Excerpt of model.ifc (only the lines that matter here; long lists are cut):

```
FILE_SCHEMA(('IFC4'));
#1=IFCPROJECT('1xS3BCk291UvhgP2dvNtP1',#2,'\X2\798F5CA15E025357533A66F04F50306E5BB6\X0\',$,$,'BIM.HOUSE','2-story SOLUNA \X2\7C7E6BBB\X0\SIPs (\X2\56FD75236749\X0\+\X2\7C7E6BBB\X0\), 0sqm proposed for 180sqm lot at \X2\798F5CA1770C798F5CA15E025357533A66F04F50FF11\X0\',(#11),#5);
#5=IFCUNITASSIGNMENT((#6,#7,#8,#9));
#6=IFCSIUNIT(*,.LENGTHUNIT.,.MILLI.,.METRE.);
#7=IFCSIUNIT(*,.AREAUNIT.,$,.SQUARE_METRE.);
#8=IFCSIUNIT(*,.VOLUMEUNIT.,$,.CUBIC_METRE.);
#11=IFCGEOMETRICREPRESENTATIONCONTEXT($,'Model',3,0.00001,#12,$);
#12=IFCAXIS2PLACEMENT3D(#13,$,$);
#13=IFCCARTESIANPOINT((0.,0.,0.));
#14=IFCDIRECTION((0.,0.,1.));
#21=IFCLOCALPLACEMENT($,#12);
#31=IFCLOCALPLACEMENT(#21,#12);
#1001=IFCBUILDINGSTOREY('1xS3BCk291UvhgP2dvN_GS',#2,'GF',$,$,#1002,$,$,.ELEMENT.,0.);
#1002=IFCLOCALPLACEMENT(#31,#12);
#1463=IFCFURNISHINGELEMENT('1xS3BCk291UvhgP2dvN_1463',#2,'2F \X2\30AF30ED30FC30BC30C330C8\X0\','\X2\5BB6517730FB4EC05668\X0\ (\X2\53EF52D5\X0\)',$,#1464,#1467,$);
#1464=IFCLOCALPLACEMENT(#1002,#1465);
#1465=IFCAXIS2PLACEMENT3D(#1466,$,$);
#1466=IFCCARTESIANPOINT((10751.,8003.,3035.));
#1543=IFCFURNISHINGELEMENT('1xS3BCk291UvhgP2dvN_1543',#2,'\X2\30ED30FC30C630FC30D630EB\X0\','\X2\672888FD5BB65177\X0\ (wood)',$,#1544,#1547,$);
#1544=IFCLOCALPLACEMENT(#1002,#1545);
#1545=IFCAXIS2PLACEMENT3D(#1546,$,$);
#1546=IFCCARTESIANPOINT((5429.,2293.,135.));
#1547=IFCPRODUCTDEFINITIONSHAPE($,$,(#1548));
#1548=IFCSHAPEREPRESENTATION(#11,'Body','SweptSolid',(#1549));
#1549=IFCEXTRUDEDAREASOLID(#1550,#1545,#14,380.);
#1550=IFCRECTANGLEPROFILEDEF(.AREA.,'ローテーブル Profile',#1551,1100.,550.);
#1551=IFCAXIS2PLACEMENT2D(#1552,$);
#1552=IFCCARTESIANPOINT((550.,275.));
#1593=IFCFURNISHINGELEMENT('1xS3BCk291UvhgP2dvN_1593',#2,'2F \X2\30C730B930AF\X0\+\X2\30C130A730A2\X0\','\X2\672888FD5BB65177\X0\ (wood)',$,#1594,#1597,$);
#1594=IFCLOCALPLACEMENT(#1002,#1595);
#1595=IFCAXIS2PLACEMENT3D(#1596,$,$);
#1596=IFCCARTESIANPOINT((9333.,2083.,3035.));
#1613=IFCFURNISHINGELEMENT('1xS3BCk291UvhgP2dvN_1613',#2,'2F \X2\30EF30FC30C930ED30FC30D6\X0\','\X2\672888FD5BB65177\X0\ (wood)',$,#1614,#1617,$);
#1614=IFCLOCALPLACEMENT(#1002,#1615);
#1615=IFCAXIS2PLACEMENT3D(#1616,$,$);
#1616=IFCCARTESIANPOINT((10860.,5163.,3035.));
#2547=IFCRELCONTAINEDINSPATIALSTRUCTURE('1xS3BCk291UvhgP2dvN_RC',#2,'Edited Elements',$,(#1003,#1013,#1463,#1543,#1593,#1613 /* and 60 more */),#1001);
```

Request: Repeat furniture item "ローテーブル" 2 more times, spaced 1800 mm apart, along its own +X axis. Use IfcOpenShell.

```python
import ifcopenshell
import ifcopenshell.api.geometry
import ifcopenshell.api.root
import ifcopenshell.util.element
import ifcopenshell.util.placement
import ifcopenshell.util.unit

model = ifcopenshell.open("model.ifc")
unit_scale = ifcopenshell.util.unit.calculate_unit_scale(model)


def reuse_history(source, copy):
    """copy_class also copies each property set's owner history, people and application; keep the originals."""
    for rel in copy.IsDefinedBy:
        if rel.is_a("IfcRelDefinesByProperties") and (history := rel.RelatingPropertyDefinition.OwnerHistory):
            rel.RelatingPropertyDefinition.OwnerHistory = source.OwnerHistory
            ifcopenshell.util.element.remove_deep2(model, history)


source = model.by_guid("1xS3BCk291UvhgP2dvN_1543")
base = ifcopenshell.util.placement.get_local_placement(source.ObjectPlacement)
step = base[:3, 0] * 1.8 / unit_scale

for i in range(1, 3):
    copy = ifcopenshell.api.root.copy_class(model, product=source)
    copy.Representation = ifcopenshell.util.element.copy_deep(
        model, source.Representation, exclude=["IfcGeometricRepresentationContext", "IfcRepresentationMap"]
    )
    reuse_history(source, copy)
    matrix = base.copy()
    matrix[:3, 3] += i * step
    print("added at", matrix[:3, 3].round(3) + 0.0)
    ifcopenshell.api.geometry.edit_object_placement(model, product=copy, matrix=matrix, is_si=False)

model.write("model_edited.ifc")
```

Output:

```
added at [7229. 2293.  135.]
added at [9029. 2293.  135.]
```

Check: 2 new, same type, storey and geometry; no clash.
